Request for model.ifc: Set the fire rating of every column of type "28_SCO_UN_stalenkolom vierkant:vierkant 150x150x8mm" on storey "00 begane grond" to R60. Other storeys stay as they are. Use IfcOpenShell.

First a look at what the model holds.

```python
import ifcopenshell
import ifcopenshell.util.element

model = ifcopenshell.open("model.ifc")
print(model.schema)
storey = next(s for s in model.by_type("IfcBuildingStorey") if s.Name == "00 begane grond")
columns = [e for e in ifcopenshell.util.element.get_decomposition(storey) if e.is_a("IfcColumn")]
seen = {}
for e in columns:
    element_type = ifcopenshell.util.element.get_type(e)
    key = (element_type.Name if element_type != e and element_type else None, ifcopenshell.util.element.get_pset(e, "Pset_ColumnCommon", "FireRating"))
    seen[key] = seen.get(key, 0) + 1
for (name, value), count in sorted(seen.items(), key=str):
    print(count, "x", name, "|", value)
```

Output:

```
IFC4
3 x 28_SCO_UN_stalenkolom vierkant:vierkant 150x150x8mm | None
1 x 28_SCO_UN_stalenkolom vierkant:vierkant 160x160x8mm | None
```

```python
import ifcopenshell
import ifcopenshell.api.pset
import ifcopenshell.util.element

model = ifcopenshell.open("model.ifc")

storey = next(s for s in model.by_type("IfcBuildingStorey") if s.Name == "00 begane grond")
columns = [e for e in ifcopenshell.util.element.get_decomposition(storey) if e.is_a("IfcColumn")]

count = 0
for e in columns:
    element_type = ifcopenshell.util.element.get_type(e)
    if element_type in (None, e) or element_type.Name != "28_SCO_UN_stalenkolom vierkant:vierkant 150x150x8mm":
        continue
    # add_pset returns the element's existing set when there is one.
    pset = ifcopenshell.api.pset.add_pset(model, product=e, name="Pset_ColumnCommon")
    ifcopenshell.api.pset.edit_pset(model, pset=pset, properties={"FireRating": "R60"})
    count += 1

print(count, "columns updated")

model.write("model_rev.ifc")
```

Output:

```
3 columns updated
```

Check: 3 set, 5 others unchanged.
